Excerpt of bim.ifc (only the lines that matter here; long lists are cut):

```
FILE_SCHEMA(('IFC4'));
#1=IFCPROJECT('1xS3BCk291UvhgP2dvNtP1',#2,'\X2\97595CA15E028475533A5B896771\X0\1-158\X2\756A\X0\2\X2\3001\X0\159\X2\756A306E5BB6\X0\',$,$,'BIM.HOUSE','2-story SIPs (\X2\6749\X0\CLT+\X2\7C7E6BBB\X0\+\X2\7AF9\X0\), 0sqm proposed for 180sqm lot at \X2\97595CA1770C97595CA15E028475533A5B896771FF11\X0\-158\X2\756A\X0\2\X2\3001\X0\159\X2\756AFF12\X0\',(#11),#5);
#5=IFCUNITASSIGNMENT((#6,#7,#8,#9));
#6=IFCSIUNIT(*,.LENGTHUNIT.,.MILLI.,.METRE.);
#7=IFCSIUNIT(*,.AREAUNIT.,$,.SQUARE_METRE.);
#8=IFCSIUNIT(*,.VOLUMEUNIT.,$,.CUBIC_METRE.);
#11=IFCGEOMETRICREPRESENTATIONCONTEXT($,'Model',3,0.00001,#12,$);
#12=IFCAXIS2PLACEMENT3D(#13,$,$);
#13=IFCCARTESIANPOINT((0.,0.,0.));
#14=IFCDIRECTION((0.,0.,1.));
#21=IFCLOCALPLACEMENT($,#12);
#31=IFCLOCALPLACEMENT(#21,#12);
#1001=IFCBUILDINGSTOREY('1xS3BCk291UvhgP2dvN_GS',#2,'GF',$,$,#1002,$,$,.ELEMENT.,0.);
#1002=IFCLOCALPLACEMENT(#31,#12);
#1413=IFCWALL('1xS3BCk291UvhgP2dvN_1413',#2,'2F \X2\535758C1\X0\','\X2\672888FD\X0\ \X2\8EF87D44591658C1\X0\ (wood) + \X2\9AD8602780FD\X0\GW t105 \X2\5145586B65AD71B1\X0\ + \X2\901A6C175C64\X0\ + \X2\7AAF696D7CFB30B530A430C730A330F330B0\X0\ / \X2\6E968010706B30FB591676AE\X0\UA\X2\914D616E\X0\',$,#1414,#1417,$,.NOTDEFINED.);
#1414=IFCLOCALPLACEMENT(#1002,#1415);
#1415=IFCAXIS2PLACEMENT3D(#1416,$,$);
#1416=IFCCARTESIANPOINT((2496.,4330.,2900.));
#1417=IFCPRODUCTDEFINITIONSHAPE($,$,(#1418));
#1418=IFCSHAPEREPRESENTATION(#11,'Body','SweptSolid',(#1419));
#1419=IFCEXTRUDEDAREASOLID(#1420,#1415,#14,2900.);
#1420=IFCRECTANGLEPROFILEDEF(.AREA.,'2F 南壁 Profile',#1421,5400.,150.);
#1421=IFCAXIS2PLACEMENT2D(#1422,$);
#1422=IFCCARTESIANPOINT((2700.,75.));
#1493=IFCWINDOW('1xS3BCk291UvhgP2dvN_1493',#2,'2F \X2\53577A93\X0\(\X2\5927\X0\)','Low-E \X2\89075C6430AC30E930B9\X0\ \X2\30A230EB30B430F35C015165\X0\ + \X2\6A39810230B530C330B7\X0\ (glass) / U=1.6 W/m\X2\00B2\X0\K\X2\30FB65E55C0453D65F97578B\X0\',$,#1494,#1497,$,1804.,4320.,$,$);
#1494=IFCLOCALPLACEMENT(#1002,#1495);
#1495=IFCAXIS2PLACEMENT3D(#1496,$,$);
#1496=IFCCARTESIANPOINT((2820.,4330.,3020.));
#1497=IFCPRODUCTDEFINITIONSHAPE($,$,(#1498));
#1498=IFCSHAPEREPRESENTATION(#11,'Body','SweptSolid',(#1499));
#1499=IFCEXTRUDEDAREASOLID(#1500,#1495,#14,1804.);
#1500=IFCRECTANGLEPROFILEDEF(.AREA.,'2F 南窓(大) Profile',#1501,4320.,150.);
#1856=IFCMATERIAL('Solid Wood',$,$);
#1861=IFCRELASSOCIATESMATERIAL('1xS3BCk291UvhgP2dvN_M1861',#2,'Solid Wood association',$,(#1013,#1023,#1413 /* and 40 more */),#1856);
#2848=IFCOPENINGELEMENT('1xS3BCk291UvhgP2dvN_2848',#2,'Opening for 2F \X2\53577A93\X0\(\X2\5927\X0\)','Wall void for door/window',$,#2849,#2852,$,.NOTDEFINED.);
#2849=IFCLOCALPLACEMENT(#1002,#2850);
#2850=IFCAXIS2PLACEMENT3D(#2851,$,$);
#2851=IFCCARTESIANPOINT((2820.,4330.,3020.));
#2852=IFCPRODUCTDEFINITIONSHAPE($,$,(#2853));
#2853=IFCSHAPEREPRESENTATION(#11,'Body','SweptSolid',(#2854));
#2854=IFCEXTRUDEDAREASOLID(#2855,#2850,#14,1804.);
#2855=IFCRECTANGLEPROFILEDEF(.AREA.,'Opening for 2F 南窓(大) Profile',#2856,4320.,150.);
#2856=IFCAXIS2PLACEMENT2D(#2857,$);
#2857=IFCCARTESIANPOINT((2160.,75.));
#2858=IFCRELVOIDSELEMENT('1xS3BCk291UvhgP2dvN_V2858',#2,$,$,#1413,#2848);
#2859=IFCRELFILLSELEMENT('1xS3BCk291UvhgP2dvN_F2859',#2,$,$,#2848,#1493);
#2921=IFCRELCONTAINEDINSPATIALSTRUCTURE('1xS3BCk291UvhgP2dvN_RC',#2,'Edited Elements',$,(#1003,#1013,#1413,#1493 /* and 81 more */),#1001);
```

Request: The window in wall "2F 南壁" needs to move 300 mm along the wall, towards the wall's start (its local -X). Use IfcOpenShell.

```python
import ifcopenshell
import ifcopenshell.api.geometry
import ifcopenshell.util.placement

model = ifcopenshell.open("bim.ifc")

window = model.by_id(1493)
opening = window.FillsVoids[0].RelatingOpeningElement
wall = opening.VoidsElements[0].RelatingBuildingElement

wall_matrix = ifcopenshell.util.placement.get_local_placement(wall.ObjectPlacement)
shift = wall_matrix[:3, 0] * -300.0
before = ifcopenshell.util.placement.get_local_placement(window.ObjectPlacement)[:3, 3].copy()

# The window is not placed relative to its opening, so move both.
for product in (opening, window):
    matrix = ifcopenshell.util.placement.get_local_placement(product.ObjectPlacement)
    matrix[:3, 3] += shift
    ifcopenshell.api.geometry.edit_object_placement(model, product=product, matrix=matrix, is_si=False)

after = ifcopenshell.util.placement.get_local_placement(window.ObjectPlacement)[:3, 3]
print("window moved by", (after - before).round(3) + 0.0)

model.write("bim_updated.ifc")
```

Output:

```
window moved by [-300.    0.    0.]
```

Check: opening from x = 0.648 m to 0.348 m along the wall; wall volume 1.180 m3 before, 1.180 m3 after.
